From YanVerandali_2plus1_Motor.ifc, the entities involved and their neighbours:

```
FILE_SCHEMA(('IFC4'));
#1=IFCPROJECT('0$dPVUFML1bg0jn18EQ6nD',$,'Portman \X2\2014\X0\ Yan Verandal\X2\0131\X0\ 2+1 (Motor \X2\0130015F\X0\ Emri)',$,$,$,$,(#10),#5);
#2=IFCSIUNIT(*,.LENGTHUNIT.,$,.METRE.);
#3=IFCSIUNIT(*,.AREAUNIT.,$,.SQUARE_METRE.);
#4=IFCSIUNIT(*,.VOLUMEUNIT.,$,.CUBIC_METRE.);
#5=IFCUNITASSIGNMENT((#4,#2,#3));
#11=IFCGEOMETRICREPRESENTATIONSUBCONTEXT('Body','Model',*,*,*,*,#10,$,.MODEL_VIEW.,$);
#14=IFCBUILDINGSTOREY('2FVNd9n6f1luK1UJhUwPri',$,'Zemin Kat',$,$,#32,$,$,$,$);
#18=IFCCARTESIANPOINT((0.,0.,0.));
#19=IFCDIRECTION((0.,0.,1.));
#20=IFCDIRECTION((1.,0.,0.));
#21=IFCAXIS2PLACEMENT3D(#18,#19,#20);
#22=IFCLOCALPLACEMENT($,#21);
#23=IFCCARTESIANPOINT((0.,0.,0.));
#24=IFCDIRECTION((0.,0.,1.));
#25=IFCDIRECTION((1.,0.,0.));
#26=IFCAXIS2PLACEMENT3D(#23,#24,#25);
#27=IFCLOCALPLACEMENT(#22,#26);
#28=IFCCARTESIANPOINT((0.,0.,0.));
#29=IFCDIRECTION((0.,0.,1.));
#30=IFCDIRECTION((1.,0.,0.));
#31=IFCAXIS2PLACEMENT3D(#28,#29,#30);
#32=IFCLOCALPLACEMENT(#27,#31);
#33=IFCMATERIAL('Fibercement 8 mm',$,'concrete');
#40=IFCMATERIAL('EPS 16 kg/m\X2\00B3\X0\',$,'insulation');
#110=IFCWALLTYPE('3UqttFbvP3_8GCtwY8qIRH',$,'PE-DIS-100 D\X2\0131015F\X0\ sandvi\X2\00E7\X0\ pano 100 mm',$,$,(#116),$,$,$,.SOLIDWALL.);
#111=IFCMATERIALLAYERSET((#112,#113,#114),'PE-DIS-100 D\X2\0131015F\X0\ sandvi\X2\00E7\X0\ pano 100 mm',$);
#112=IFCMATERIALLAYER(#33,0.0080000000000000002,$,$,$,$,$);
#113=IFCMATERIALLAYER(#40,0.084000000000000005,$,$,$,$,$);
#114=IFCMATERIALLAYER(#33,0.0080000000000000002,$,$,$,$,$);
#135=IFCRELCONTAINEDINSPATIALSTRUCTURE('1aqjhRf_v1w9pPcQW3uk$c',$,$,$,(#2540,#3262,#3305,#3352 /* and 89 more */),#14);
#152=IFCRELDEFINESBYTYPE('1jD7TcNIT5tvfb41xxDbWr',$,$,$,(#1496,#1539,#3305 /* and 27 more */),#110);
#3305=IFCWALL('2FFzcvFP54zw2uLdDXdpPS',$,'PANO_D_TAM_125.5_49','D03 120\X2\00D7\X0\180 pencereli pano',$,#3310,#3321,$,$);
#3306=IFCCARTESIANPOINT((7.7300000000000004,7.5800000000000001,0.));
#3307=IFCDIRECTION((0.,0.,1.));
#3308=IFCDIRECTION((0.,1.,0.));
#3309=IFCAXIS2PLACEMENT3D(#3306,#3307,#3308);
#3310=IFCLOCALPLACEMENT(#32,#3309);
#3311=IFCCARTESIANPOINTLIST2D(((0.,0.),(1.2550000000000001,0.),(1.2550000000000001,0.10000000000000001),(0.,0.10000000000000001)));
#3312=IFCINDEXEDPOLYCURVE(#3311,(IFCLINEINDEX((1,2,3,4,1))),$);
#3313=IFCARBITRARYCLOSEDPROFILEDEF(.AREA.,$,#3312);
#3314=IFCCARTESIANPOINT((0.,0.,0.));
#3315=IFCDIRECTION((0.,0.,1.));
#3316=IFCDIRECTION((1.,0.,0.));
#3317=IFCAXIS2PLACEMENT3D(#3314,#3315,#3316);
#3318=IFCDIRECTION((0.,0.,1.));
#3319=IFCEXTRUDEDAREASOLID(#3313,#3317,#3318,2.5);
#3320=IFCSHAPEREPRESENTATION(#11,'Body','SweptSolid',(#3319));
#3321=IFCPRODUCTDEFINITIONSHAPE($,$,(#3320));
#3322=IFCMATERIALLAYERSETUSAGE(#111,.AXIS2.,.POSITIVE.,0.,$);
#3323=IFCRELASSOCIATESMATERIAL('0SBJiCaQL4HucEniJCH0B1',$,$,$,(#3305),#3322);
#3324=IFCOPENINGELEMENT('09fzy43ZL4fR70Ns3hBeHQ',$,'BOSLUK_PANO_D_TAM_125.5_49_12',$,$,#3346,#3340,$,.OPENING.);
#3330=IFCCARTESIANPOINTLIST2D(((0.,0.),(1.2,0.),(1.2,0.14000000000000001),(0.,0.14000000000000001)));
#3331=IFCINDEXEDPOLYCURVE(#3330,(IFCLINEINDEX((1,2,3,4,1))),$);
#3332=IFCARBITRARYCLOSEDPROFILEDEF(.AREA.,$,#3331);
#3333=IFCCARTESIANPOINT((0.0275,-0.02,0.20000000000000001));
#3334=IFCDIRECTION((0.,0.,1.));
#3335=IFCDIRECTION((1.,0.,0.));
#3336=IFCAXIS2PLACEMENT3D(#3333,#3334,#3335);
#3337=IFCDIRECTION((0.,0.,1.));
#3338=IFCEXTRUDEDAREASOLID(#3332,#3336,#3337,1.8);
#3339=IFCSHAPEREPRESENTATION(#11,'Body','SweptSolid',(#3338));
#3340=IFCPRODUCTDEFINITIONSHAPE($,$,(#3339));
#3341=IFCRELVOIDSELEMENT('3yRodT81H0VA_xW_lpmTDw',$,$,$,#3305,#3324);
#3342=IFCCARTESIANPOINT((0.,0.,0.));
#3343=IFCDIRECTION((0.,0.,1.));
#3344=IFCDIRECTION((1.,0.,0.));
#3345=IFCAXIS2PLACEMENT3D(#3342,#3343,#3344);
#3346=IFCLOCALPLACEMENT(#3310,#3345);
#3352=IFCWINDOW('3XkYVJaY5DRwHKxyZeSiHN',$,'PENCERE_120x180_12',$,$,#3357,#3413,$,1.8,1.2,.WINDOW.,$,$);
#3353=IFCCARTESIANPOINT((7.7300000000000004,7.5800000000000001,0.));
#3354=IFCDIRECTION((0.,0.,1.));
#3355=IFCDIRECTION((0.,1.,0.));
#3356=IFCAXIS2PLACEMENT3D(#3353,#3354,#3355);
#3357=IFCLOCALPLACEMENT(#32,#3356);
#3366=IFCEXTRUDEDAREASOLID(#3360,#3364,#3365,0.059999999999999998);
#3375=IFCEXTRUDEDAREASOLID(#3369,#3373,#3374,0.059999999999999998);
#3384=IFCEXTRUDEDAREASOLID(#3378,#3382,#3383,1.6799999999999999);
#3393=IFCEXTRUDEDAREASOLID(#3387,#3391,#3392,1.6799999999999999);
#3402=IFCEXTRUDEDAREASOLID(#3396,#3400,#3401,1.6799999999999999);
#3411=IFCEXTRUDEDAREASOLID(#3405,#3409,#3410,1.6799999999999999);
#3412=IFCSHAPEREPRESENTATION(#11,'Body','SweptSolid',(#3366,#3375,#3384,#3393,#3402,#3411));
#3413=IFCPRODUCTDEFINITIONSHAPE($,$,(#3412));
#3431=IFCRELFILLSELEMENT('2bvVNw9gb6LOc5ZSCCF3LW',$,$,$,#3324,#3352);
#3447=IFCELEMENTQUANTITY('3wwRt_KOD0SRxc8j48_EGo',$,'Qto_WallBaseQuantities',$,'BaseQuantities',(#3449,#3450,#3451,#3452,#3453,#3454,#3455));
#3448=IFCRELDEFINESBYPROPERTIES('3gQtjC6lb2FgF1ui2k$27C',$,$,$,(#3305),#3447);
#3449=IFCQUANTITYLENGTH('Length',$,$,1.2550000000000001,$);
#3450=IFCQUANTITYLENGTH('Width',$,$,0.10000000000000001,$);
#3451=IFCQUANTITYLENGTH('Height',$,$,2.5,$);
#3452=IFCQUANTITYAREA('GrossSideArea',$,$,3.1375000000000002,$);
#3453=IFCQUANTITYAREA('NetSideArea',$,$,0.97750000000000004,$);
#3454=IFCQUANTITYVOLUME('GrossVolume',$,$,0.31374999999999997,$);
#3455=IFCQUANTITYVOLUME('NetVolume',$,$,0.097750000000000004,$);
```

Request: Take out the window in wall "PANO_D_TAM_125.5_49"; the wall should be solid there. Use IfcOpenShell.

```python
import ifcopenshell
import ifcopenshell.api.feature
import ifcopenshell.api.pset
import ifcopenshell.api.root
import ifcopenshell.geom
import ifcopenshell.util.element
import ifcopenshell.util.shape
import ifcopenshell.util.unit

model = ifcopenshell.open("YanVerandali_2plus1_Motor.ifc")
area_scale = ifcopenshell.util.unit.calculate_unit_scale(model, "AREAUNIT")
volume_scale = ifcopenshell.util.unit.calculate_unit_scale(model, "VOLUMEUNIT")
settings = ifcopenshell.geom.settings()


def volume(element):
    """Net volume in cubic metres, openings subtracted."""
    shape = ifcopenshell.geom.create_shape(settings, element)
    return ifcopenshell.util.shape.get_volume(shape.geometry)


window = model.by_guid("3XkYVJaY5DRwHKxyZeSiHN")
opening = window.FillsVoids[0].RelatingOpeningElement
wall = opening.VoidsElements[0].RelatingBuildingElement
before = volume(wall)

ifcopenshell.api.root.remove_product(model, product=window)
ifcopenshell.api.feature.remove_feature(model, feature=opening)

after = volume(wall)
thickness = 0.1  # wall thickness in metres

# Update the wall's stored quantities.
qto = model.by_id(ifcopenshell.util.element.get_pset(wall, "Qto_WallBaseQuantities", should_inherit=False)["id"])
ifcopenshell.api.pset.edit_qto(model, qto=qto, properties={
    "NetSideArea": after / thickness / area_scale,
    "NetVolume": after / volume_scale,
})

print(f"wall volume {before:.3f} -> {after:.3f} m3")

model.write("YanVerandali_2plus1_Motor-out.ifc")
```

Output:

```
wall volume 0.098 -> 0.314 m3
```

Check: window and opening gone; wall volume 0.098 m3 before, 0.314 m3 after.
